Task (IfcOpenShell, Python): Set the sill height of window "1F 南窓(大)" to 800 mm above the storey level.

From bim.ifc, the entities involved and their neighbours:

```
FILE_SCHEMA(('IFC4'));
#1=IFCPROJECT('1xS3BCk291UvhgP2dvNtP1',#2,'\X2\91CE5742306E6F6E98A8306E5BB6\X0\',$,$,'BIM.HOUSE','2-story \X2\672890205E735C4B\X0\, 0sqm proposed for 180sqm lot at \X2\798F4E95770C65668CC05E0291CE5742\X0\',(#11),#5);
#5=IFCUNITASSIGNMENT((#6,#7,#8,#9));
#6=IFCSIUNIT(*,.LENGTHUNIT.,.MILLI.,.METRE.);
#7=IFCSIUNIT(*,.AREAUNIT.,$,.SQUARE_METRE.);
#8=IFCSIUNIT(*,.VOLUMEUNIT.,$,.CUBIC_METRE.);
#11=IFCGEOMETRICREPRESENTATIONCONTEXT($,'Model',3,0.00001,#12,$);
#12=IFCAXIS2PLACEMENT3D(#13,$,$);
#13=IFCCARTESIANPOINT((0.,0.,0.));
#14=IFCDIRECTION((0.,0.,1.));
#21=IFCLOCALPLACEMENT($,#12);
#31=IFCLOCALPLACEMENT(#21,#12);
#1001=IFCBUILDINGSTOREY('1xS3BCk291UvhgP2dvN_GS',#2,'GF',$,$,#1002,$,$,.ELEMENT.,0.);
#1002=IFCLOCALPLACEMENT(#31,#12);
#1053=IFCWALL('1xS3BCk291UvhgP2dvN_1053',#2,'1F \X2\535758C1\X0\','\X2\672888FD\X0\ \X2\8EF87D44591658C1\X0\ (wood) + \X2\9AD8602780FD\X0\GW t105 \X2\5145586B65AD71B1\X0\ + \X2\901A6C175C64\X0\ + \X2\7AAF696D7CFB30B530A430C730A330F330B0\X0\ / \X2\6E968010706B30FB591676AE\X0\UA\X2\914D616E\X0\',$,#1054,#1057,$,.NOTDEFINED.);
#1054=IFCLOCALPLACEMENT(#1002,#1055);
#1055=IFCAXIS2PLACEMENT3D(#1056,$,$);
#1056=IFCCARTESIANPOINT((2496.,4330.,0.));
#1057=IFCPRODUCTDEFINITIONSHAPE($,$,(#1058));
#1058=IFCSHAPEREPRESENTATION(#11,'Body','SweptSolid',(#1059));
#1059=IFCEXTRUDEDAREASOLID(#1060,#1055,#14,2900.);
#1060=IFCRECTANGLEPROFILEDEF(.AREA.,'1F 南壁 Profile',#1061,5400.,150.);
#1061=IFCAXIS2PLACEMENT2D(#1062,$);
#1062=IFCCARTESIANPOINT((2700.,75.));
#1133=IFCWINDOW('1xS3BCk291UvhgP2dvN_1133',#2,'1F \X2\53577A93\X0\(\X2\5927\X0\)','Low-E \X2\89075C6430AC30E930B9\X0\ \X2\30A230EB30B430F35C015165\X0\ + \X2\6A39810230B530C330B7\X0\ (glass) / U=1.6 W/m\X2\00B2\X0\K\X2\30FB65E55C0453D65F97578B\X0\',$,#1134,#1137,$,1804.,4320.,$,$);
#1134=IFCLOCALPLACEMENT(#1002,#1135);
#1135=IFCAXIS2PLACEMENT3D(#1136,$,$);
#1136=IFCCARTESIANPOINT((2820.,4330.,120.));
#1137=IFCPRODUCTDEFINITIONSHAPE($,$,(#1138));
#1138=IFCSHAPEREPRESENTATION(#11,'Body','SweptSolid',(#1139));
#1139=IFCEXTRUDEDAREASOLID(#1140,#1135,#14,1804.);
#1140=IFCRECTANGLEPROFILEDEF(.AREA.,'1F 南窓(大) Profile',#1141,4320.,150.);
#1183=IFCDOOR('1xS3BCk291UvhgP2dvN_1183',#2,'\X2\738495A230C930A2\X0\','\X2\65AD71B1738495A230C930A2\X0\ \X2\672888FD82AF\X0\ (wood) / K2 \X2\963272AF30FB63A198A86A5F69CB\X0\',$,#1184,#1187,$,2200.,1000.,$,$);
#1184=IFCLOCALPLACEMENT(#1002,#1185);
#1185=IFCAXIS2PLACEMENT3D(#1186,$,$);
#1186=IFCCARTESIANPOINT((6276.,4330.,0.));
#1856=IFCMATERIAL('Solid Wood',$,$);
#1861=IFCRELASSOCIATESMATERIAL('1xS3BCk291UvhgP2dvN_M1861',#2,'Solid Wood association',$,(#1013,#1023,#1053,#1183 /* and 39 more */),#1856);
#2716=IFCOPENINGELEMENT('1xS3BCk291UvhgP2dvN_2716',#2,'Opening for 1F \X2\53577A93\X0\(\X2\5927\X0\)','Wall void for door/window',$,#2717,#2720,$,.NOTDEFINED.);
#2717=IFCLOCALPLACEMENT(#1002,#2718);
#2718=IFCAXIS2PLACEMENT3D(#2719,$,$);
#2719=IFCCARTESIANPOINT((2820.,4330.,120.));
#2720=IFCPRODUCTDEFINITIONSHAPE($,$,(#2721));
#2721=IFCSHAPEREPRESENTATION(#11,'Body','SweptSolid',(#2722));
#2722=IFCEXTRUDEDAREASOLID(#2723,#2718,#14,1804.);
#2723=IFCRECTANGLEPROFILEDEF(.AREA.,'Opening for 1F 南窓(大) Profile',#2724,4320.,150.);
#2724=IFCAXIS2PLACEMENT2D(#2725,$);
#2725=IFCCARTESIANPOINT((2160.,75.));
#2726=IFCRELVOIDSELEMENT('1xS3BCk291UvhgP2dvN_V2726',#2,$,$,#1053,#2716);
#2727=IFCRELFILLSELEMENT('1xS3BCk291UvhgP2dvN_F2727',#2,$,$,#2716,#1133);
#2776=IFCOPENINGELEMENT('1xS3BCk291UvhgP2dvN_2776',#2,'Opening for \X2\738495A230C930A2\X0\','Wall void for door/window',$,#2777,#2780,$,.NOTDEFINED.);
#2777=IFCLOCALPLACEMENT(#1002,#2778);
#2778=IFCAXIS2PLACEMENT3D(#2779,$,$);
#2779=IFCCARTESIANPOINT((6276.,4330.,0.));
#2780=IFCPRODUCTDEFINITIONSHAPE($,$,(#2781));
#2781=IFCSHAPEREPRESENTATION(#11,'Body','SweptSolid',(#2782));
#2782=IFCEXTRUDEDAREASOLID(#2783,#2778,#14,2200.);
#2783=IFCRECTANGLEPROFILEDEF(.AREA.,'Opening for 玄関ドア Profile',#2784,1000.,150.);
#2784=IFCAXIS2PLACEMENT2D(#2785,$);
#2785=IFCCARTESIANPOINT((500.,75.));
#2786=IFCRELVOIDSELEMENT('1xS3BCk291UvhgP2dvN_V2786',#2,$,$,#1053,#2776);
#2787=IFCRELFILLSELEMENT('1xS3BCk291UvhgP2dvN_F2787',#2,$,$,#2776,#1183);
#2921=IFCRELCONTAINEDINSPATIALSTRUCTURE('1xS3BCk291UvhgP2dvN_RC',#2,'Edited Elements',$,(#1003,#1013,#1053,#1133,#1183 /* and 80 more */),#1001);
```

```python
import numpy as np
import ifcopenshell
import ifcopenshell.api.geometry
import ifcopenshell.geom
import ifcopenshell.util.element
import ifcopenshell.util.placement
import ifcopenshell.util.shape
import ifcopenshell.util.unit

model = ifcopenshell.open("bim.ifc")
unit_scale = ifcopenshell.util.unit.calculate_unit_scale(model)

window = model.by_id(1133)
opening = window.FillsVoids[0].RelatingOpeningElement
storey = ifcopenshell.util.element.get_container(window, ifc_class="IfcBuildingStorey")
level = ifcopenshell.util.placement.get_local_placement(storey.ObjectPlacement)[2, 3]

# The opening's origin need not be at the sill, so measure its lowest point.
shape = ifcopenshell.geom.create_shape(ifcopenshell.geom.settings(), opening)
bottom = ifcopenshell.util.shape.get_shape_bottom_elevation(shape, shape.geometry) / unit_scale
dz = level + 800.0 - bottom

shift = np.array([0.0, 0.0, dz])
# The window is not placed relative to its opening, so move both.
for product in (opening, window):
    matrix = ifcopenshell.util.placement.get_local_placement(product.ObjectPlacement)
    matrix[:3, 3] += shift
    ifcopenshell.api.geometry.edit_object_placement(model, product=product, matrix=matrix, is_si=False)

print(f"moved by {dz * unit_scale:+.3f} m")

model.write("bim_updated.ifc")
```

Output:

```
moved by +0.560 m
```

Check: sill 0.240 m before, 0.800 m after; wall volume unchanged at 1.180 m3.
